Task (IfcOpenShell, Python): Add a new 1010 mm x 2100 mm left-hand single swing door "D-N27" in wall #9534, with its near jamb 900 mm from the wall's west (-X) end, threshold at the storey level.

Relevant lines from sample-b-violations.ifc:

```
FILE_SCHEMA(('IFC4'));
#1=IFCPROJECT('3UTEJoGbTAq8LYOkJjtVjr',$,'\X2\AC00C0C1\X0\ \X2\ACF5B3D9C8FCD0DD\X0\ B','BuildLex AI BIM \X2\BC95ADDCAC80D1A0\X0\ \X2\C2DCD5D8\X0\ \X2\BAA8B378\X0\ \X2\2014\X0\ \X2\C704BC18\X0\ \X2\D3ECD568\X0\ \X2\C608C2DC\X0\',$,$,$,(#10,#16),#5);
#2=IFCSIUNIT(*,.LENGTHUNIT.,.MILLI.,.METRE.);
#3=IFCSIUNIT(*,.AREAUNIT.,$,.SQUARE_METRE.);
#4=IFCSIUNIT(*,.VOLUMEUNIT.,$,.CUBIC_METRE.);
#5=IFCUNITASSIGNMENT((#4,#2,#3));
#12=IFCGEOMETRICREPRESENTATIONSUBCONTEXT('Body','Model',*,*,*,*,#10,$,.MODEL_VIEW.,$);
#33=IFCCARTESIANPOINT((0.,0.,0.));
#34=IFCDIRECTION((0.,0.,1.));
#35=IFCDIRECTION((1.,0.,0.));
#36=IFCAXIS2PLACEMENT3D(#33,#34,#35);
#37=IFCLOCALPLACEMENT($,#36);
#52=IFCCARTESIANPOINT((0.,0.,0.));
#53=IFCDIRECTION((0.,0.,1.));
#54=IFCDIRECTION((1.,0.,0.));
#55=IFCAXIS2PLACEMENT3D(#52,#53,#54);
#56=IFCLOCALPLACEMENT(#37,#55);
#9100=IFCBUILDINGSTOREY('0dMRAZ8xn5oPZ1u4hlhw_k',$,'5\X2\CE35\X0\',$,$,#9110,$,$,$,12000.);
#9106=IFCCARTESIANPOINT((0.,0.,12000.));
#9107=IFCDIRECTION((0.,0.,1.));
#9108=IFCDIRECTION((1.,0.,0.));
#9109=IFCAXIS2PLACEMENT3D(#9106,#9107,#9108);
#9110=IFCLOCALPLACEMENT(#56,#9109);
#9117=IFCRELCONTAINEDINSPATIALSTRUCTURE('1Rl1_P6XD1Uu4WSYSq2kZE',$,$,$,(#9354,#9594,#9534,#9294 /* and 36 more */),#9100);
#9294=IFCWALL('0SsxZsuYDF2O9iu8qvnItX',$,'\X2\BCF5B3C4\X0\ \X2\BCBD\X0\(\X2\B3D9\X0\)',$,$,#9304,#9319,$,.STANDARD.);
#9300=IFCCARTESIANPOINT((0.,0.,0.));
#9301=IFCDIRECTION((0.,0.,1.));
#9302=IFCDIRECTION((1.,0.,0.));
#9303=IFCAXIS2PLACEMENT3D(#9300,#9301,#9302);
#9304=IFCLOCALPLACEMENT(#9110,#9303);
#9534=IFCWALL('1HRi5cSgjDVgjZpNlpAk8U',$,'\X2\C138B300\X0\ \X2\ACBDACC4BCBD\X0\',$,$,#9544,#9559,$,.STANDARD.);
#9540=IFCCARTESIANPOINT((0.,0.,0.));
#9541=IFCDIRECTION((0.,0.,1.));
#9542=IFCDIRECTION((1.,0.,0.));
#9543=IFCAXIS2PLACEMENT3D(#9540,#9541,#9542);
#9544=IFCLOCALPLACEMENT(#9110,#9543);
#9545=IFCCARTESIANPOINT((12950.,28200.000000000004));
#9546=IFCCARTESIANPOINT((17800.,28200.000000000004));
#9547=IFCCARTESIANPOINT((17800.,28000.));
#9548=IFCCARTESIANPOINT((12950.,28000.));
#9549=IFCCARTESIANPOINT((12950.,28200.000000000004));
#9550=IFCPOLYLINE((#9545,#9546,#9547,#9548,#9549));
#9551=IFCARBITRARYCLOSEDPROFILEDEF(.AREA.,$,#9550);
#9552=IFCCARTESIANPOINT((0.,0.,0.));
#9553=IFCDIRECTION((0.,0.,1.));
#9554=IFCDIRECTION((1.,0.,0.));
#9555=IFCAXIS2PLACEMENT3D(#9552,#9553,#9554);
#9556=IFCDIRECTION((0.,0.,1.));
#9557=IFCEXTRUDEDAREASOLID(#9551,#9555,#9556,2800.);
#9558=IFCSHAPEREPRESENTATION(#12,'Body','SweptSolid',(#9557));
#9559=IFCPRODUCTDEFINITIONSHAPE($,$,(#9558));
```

```python
import numpy as np
import ifcopenshell
import ifcopenshell.api.feature
import ifcopenshell.api.geometry
import ifcopenshell.api.root
import ifcopenshell.api.spatial
import ifcopenshell.geom
import ifcopenshell.util.element
import ifcopenshell.util.placement
import ifcopenshell.util.representation
import ifcopenshell.util.shape
import ifcopenshell.util.unit

model = ifcopenshell.open("sample-b-violations.ifc")
unit_scale = ifcopenshell.util.unit.calculate_unit_scale(model)
settings = ifcopenshell.geom.settings()


def volume(element):
    """Net volume in cubic metres, openings subtracted."""
    shape = ifcopenshell.geom.create_shape(settings, element)
    return ifcopenshell.util.shape.get_volume(shape.geometry)


wall = model.by_guid("1HRi5cSgjDVgjZpNlpAk8U")
storey = ifcopenshell.util.element.get_container(wall, ifc_class="IfcBuildingStorey")
context = ifcopenshell.util.representation.get_context(model, "Model", "Body", "MODEL_VIEW")
before = volume(wall)

width, height, from_end, sill = 1.01, 2.1, 0.9, 0.0  # metres

# The wall runs along its own X axis, and the end named is its -X end.
wall_shape = ifcopenshell.geom.create_shape(settings, wall)
x, y, z = ifcopenshell.util.shape.get_vertices(wall_shape.geometry).T
start = x.min() + from_end
face, thickness = float(y.min()), float(y.max() - y.min())
wall_matrix = ifcopenshell.util.placement.get_local_placement(wall.ObjectPlacement)
level = ifcopenshell.util.placement.get_local_placement(storey.ObjectPlacement)[2, 3]


def in_wall(x, y):
    """Placement at x, y metres in the wall's axes, at sill height."""
    matrix = wall_matrix.copy()
    matrix[:, 3] = wall_matrix @ np.array([x / unit_scale, y / unit_scale, 0.0, 1.0])
    matrix[2, 3] = level + sill / unit_scale
    return matrix


# Opening: a box that overshoots both wall faces by 50 mm.
opening = ifcopenshell.api.root.create_entity(model, ifc_class="IfcOpeningElement", predefined_type="OPENING")
box = ifcopenshell.api.geometry.add_wall_representation(
    model, context=context, length=width, height=height, thickness=thickness + 0.1
)
ifcopenshell.api.geometry.assign_representation(model, product=opening, representation=box)
ifcopenshell.api.geometry.edit_object_placement(model, product=opening, matrix=in_wall(start, face - 0.05), is_si=False)
ifcopenshell.api.feature.add_feature(model, feature=opening, element=wall)

door = ifcopenshell.api.root.create_entity(model, ifc_class="IfcDoor", name="D-N27", predefined_type="DOOR")
door.OverallWidth, door.OverallHeight = width / unit_scale, height / unit_scale
door.OperationType = "SINGLE_SWING_LEFT"
body = ifcopenshell.api.geometry.add_door_representation(
    model,
    context=context,
    overall_width=door.OverallWidth,
    overall_height=door.OverallHeight,
    operation_type="SINGLE_SWING_LEFT",
    lining_properties={"LiningDepth": thickness / unit_scale, "ThresholdDepth": thickness / unit_scale},
)
ifcopenshell.api.geometry.assign_representation(model, product=door, representation=body)
ifcopenshell.api.spatial.assign_container(model, products=[door], relating_structure=storey)
ifcopenshell.api.feature.add_filling(model, opening=opening, element=door)

# The lining spans the wall, so the door starts at the wall face.
ifcopenshell.api.geometry.edit_object_placement(model, product=door, matrix=in_wall(start, face), is_si=False)

after = volume(wall)

print(f"wall volume {before:.3f} -> {after:.3f} m3")

model.write("sample-b-violations_rev.ifc")
```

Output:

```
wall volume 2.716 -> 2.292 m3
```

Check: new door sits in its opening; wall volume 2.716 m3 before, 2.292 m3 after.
